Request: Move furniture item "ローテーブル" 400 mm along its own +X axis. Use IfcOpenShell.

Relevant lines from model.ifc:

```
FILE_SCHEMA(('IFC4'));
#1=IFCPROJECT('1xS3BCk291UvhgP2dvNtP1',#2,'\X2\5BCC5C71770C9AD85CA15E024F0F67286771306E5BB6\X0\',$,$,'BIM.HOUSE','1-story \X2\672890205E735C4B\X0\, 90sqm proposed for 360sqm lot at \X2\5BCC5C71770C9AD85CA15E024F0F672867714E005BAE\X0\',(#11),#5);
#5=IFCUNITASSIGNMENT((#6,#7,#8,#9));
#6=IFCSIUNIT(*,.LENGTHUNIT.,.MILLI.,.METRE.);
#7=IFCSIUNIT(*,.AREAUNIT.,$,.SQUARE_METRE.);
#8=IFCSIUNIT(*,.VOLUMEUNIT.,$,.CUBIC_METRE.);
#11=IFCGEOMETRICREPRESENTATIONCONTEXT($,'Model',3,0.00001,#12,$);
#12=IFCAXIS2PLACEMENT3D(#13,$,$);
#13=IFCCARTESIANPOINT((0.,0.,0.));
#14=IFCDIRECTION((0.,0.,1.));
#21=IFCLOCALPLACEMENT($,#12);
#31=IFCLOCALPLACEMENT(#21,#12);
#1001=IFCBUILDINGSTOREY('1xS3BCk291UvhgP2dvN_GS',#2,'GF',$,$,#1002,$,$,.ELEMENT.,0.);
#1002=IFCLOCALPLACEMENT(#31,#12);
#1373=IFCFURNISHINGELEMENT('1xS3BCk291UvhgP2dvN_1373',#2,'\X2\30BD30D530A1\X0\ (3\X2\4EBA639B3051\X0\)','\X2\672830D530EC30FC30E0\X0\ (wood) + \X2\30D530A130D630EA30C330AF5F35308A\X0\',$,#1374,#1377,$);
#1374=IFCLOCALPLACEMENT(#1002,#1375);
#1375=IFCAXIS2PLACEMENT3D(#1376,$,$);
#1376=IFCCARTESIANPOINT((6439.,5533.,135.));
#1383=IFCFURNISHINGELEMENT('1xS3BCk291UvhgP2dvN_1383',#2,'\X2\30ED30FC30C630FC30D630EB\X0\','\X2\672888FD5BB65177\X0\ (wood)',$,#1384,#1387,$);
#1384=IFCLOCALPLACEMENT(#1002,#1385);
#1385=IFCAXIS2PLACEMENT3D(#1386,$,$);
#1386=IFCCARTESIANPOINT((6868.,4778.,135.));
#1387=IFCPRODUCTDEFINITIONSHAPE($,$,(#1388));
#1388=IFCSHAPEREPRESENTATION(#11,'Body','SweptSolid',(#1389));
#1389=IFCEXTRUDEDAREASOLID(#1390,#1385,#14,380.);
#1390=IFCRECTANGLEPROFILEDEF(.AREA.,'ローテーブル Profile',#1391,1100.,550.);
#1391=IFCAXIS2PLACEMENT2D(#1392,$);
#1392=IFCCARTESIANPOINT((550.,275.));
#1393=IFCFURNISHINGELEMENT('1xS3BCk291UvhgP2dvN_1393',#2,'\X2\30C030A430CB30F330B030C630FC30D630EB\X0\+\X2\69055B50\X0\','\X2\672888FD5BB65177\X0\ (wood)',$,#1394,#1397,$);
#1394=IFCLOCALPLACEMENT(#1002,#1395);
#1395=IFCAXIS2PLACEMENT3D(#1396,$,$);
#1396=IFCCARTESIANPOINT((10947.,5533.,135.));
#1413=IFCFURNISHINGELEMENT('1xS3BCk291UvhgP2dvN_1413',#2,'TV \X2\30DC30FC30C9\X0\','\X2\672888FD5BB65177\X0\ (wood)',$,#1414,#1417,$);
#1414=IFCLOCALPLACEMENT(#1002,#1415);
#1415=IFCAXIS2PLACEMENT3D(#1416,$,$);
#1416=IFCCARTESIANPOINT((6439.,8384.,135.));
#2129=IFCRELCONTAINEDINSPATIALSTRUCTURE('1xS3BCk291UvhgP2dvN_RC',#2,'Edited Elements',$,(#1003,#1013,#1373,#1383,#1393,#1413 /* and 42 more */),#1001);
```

```python
import ifcopenshell
import ifcopenshell.api.geometry
import ifcopenshell.util.placement

model = ifcopenshell.open("model.ifc")

item = model.by_guid("1xS3BCk291UvhgP2dvN_1383")
matrix = ifcopenshell.util.placement.get_local_placement(item.ObjectPlacement)
matrix[:3, 3] += matrix[:3, 0] * 400.0
ifcopenshell.api.geometry.edit_object_placement(model, product=item, matrix=matrix, is_si=False)

print(ifcopenshell.util.placement.get_local_placement(item.ObjectPlacement).round(3) + 0.0)

model.write("model_rev.ifc")
```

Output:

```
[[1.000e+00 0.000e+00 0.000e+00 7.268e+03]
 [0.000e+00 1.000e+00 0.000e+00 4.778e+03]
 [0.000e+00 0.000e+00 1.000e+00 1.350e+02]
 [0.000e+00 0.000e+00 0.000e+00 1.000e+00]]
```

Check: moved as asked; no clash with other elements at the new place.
